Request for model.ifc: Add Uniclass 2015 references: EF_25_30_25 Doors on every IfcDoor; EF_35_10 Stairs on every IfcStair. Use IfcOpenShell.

First a look at what the model holds.

```python
import ifcopenshell

model = ifcopenshell.open("model.ifc")
print(model.schema)
print("classifications:", [c.Name for c in model.by_type("IfcClassification")])
for ifc_class in ("IfcDoor", "IfcRoof", "IfcStair", "IfcWall", "IfcWindow"):
    print(ifc_class, len(model.by_type(ifc_class)))
```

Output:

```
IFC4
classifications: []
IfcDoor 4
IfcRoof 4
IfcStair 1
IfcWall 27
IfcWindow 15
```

```python
import ifcopenshell
import ifcopenshell.api.classification

model = ifcopenshell.open("model.ifc")

system = ifcopenshell.api.classification.add_classification(model, classification="Uniclass 2015")

codes = {
    "IfcDoor": ("EF_25_30_25", "Doors"),
    "IfcStair": ("EF_35_10", "Stairs"),
}
for ifc_class, (code, name) in codes.items():
    products = model.by_type(ifc_class)
    ifcopenshell.api.classification.add_reference(
        model, products=products, classification=system, identification=code, name=name
    )
    print(code, len(products))

model.write("model_updated.ifc")
```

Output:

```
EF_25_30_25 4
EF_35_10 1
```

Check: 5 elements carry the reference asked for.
